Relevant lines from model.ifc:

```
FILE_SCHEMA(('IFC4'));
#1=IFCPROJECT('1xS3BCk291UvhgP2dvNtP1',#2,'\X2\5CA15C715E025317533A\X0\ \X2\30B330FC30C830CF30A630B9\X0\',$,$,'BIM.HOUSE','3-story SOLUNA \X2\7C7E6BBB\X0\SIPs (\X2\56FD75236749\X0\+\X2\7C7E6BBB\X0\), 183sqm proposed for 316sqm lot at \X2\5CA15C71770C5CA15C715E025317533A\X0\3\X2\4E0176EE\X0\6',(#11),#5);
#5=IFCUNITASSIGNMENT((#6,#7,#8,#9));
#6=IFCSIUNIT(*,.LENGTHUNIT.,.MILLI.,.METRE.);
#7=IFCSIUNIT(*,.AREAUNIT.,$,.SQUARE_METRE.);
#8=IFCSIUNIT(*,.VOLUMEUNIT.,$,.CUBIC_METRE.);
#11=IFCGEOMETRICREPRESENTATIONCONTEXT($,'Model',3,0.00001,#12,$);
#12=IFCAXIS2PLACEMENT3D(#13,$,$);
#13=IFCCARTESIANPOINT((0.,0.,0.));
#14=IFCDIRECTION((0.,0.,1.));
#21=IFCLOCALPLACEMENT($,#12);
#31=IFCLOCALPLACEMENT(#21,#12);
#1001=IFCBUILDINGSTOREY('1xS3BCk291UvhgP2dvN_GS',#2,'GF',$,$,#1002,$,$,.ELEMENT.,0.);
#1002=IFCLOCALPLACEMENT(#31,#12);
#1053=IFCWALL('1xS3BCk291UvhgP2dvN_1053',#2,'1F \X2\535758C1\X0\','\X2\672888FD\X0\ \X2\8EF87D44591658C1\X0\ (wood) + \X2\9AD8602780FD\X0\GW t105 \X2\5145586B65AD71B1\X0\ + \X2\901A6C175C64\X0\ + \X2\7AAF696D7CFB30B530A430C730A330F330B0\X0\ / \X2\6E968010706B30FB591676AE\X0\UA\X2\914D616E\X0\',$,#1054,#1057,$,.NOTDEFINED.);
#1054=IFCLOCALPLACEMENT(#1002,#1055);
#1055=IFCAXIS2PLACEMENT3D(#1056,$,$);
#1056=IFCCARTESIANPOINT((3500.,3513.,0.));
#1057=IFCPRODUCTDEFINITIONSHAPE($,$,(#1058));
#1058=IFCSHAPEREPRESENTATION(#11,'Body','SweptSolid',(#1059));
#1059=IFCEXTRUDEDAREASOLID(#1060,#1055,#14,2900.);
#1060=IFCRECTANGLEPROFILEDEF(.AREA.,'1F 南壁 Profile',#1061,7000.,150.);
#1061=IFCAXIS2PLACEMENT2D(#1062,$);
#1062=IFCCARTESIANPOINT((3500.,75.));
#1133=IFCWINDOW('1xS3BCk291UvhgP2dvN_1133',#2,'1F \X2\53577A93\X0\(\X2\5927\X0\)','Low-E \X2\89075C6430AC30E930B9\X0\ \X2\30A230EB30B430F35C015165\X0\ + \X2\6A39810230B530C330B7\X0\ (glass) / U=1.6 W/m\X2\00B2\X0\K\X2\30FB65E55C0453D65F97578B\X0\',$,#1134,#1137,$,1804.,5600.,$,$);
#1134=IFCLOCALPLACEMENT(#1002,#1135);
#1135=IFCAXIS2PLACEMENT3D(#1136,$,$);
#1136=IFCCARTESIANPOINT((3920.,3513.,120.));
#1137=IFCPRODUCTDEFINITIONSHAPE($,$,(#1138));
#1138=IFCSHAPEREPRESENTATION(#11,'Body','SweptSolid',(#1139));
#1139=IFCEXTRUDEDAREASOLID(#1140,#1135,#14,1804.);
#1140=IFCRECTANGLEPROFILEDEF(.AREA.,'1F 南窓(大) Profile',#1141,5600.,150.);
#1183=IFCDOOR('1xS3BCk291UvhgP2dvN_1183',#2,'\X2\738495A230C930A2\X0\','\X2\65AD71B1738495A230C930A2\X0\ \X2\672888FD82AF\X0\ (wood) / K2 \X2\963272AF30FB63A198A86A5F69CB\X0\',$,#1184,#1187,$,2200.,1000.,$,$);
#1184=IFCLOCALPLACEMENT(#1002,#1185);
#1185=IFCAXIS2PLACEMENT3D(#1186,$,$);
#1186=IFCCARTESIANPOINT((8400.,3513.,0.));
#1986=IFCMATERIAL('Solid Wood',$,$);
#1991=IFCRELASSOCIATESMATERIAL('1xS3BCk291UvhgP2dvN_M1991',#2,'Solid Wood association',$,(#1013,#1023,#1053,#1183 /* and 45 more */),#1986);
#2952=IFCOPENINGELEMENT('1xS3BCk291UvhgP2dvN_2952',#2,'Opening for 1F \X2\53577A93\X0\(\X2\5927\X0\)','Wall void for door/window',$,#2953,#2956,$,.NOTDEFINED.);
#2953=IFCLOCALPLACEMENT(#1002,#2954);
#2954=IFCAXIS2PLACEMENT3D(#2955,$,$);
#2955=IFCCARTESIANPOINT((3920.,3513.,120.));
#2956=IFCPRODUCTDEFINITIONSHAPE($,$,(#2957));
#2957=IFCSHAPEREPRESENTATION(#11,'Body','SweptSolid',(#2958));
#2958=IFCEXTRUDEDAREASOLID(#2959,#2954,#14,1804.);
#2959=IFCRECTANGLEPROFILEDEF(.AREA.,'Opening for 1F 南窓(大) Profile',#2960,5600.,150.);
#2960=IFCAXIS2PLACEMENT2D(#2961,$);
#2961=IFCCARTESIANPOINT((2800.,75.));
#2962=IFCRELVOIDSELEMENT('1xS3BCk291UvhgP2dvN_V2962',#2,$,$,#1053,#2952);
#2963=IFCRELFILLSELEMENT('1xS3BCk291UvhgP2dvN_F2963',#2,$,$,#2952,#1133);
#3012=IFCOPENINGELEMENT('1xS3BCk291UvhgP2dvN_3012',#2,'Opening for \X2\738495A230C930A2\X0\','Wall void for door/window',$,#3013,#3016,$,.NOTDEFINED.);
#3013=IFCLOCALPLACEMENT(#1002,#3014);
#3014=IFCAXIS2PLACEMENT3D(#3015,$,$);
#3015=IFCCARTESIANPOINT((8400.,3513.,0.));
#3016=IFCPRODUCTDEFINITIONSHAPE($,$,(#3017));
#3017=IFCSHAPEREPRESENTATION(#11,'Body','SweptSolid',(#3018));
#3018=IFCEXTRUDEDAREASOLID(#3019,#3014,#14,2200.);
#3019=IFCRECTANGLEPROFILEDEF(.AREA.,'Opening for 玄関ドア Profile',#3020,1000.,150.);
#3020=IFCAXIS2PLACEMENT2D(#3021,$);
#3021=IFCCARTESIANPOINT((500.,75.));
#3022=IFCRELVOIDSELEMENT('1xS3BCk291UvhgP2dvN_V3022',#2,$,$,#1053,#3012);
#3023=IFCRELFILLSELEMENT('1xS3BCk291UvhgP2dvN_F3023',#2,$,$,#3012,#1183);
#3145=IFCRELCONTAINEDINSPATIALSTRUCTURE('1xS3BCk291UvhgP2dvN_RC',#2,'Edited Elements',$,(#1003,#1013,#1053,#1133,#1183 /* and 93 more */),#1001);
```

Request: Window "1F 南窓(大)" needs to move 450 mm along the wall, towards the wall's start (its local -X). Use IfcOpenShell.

```python
import ifcopenshell
import ifcopenshell.api.geometry
import ifcopenshell.util.placement

model = ifcopenshell.open("model.ifc")

window = model.by_guid("1xS3BCk291UvhgP2dvN_1133")
opening = window.FillsVoids[0].RelatingOpeningElement
wall = opening.VoidsElements[0].RelatingBuildingElement

wall_matrix = ifcopenshell.util.placement.get_local_placement(wall.ObjectPlacement)
shift = wall_matrix[:3, 0] * -450.0
before = ifcopenshell.util.placement.get_local_placement(window.ObjectPlacement)[:3, 3].copy()

# The window is not placed relative to its opening, so move both.
for product in (opening, window):
    matrix = ifcopenshell.util.placement.get_local_placement(product.ObjectPlacement)
    matrix[:3, 3] += shift
    ifcopenshell.api.geometry.edit_object_placement(model, product=product, matrix=matrix, is_si=False)

after = ifcopenshell.util.placement.get_local_placement(window.ObjectPlacement)[:3, 3]
print("window moved by", (after - before).round(3) + 0.0)

model.write("model_rev.ifc")
```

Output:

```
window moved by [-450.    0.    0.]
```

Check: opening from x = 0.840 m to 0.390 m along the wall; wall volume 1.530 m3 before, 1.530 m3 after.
